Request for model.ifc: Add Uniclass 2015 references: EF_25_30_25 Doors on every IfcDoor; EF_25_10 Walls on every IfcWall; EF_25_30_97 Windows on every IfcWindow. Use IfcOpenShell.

First a look at what the model holds.

```python
import ifcopenshell

model = ifcopenshell.open("model.ifc")
print(model.schema)
print("classifications:", [c.Name for c in model.by_type("IfcClassification")])
for ifc_class in ("IfcDoor", "IfcRoof", "IfcStair", "IfcWall", "IfcWindow"):
    print(ifc_class, len(model.by_type(ifc_class)))
```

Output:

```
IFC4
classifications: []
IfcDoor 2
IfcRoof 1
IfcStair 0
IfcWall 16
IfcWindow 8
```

```python
import ifcopenshell
import ifcopenshell.api.classification

model = ifcopenshell.open("model.ifc")

system = ifcopenshell.api.classification.add_classification(model, classification="Uniclass 2015")

codes = {
    "IfcDoor": ("EF_25_30_25", "Doors"),
    "IfcWall": ("EF_25_10", "Walls"),
    "IfcWindow": ("EF_25_30_97", "Windows"),
}
for ifc_class, (code, name) in codes.items():
    products = model.by_type(ifc_class)
    ifcopenshell.api.classification.add_reference(
        model, products=products, classification=system, identification=code, name=name
    )
    print(code, len(products))

model.write("model_rev.ifc")
```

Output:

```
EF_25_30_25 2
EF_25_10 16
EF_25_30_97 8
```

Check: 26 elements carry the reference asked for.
